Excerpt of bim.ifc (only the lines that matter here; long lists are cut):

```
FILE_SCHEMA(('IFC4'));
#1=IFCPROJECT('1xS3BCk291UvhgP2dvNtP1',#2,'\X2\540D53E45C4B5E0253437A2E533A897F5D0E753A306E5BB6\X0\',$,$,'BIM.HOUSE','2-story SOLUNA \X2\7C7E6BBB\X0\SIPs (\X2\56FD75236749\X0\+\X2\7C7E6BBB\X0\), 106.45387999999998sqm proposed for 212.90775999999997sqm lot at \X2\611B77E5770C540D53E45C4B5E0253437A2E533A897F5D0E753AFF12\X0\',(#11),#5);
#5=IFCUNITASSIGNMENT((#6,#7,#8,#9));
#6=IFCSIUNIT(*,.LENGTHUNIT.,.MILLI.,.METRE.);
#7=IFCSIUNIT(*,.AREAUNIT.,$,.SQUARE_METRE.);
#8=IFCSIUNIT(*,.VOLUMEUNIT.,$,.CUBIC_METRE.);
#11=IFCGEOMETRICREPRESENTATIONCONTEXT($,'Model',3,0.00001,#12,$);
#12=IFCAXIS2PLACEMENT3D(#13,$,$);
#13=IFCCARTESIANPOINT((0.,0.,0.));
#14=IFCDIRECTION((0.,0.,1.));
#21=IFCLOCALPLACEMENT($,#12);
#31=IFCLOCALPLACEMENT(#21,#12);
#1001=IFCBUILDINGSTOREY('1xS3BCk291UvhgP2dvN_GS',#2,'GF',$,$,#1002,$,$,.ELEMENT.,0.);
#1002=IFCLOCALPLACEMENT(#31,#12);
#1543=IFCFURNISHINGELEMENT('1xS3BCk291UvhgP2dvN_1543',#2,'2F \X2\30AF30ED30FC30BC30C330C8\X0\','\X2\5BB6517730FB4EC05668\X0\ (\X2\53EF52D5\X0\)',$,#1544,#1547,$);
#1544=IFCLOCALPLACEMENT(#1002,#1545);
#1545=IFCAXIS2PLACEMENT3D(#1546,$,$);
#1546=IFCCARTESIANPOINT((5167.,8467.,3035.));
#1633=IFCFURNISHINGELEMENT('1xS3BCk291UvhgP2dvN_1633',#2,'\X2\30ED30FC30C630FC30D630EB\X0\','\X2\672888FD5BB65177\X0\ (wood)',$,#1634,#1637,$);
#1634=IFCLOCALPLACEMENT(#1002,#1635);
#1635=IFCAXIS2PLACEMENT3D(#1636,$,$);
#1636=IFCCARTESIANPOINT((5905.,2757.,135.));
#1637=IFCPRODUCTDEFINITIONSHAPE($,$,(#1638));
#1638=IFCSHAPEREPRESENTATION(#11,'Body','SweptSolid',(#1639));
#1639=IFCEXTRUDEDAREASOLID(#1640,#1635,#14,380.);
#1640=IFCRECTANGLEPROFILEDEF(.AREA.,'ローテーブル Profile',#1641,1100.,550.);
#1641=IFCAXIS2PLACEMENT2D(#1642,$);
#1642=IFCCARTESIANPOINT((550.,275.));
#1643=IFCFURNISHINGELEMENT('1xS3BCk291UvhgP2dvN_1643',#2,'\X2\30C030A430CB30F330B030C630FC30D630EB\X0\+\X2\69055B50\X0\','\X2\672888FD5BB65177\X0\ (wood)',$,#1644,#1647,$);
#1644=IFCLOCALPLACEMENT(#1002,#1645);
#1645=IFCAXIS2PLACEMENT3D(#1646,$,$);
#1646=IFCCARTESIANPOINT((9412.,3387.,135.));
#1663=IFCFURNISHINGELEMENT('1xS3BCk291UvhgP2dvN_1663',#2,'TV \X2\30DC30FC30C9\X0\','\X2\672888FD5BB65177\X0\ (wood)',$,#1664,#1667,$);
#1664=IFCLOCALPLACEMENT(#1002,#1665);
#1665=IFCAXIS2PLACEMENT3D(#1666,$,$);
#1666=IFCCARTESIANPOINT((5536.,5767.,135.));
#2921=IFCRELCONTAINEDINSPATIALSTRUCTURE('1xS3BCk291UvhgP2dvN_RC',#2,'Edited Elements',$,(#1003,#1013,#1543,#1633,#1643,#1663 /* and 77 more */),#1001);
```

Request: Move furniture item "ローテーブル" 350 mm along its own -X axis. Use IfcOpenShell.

```python
import ifcopenshell
import ifcopenshell.api.geometry
import ifcopenshell.util.placement
import ifcopenshell.util.unit

model = ifcopenshell.open("bim.ifc")
unit_scale = ifcopenshell.util.unit.calculate_unit_scale(model)

item = model.by_id(1633)
matrix = ifcopenshell.util.placement.get_local_placement(item.ObjectPlacement)
matrix[:3, 3] -= matrix[:3, 0] * 0.35 / unit_scale
ifcopenshell.api.geometry.edit_object_placement(model, product=item, matrix=matrix, is_si=False)

print(ifcopenshell.util.placement.get_local_placement(item.ObjectPlacement).round(3) + 0.0)

model.write("bim-out.ifc")
```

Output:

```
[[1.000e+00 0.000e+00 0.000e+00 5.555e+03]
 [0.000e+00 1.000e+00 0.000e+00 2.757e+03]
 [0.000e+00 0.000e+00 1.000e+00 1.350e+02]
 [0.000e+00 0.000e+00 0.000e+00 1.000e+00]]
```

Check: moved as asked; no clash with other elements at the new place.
